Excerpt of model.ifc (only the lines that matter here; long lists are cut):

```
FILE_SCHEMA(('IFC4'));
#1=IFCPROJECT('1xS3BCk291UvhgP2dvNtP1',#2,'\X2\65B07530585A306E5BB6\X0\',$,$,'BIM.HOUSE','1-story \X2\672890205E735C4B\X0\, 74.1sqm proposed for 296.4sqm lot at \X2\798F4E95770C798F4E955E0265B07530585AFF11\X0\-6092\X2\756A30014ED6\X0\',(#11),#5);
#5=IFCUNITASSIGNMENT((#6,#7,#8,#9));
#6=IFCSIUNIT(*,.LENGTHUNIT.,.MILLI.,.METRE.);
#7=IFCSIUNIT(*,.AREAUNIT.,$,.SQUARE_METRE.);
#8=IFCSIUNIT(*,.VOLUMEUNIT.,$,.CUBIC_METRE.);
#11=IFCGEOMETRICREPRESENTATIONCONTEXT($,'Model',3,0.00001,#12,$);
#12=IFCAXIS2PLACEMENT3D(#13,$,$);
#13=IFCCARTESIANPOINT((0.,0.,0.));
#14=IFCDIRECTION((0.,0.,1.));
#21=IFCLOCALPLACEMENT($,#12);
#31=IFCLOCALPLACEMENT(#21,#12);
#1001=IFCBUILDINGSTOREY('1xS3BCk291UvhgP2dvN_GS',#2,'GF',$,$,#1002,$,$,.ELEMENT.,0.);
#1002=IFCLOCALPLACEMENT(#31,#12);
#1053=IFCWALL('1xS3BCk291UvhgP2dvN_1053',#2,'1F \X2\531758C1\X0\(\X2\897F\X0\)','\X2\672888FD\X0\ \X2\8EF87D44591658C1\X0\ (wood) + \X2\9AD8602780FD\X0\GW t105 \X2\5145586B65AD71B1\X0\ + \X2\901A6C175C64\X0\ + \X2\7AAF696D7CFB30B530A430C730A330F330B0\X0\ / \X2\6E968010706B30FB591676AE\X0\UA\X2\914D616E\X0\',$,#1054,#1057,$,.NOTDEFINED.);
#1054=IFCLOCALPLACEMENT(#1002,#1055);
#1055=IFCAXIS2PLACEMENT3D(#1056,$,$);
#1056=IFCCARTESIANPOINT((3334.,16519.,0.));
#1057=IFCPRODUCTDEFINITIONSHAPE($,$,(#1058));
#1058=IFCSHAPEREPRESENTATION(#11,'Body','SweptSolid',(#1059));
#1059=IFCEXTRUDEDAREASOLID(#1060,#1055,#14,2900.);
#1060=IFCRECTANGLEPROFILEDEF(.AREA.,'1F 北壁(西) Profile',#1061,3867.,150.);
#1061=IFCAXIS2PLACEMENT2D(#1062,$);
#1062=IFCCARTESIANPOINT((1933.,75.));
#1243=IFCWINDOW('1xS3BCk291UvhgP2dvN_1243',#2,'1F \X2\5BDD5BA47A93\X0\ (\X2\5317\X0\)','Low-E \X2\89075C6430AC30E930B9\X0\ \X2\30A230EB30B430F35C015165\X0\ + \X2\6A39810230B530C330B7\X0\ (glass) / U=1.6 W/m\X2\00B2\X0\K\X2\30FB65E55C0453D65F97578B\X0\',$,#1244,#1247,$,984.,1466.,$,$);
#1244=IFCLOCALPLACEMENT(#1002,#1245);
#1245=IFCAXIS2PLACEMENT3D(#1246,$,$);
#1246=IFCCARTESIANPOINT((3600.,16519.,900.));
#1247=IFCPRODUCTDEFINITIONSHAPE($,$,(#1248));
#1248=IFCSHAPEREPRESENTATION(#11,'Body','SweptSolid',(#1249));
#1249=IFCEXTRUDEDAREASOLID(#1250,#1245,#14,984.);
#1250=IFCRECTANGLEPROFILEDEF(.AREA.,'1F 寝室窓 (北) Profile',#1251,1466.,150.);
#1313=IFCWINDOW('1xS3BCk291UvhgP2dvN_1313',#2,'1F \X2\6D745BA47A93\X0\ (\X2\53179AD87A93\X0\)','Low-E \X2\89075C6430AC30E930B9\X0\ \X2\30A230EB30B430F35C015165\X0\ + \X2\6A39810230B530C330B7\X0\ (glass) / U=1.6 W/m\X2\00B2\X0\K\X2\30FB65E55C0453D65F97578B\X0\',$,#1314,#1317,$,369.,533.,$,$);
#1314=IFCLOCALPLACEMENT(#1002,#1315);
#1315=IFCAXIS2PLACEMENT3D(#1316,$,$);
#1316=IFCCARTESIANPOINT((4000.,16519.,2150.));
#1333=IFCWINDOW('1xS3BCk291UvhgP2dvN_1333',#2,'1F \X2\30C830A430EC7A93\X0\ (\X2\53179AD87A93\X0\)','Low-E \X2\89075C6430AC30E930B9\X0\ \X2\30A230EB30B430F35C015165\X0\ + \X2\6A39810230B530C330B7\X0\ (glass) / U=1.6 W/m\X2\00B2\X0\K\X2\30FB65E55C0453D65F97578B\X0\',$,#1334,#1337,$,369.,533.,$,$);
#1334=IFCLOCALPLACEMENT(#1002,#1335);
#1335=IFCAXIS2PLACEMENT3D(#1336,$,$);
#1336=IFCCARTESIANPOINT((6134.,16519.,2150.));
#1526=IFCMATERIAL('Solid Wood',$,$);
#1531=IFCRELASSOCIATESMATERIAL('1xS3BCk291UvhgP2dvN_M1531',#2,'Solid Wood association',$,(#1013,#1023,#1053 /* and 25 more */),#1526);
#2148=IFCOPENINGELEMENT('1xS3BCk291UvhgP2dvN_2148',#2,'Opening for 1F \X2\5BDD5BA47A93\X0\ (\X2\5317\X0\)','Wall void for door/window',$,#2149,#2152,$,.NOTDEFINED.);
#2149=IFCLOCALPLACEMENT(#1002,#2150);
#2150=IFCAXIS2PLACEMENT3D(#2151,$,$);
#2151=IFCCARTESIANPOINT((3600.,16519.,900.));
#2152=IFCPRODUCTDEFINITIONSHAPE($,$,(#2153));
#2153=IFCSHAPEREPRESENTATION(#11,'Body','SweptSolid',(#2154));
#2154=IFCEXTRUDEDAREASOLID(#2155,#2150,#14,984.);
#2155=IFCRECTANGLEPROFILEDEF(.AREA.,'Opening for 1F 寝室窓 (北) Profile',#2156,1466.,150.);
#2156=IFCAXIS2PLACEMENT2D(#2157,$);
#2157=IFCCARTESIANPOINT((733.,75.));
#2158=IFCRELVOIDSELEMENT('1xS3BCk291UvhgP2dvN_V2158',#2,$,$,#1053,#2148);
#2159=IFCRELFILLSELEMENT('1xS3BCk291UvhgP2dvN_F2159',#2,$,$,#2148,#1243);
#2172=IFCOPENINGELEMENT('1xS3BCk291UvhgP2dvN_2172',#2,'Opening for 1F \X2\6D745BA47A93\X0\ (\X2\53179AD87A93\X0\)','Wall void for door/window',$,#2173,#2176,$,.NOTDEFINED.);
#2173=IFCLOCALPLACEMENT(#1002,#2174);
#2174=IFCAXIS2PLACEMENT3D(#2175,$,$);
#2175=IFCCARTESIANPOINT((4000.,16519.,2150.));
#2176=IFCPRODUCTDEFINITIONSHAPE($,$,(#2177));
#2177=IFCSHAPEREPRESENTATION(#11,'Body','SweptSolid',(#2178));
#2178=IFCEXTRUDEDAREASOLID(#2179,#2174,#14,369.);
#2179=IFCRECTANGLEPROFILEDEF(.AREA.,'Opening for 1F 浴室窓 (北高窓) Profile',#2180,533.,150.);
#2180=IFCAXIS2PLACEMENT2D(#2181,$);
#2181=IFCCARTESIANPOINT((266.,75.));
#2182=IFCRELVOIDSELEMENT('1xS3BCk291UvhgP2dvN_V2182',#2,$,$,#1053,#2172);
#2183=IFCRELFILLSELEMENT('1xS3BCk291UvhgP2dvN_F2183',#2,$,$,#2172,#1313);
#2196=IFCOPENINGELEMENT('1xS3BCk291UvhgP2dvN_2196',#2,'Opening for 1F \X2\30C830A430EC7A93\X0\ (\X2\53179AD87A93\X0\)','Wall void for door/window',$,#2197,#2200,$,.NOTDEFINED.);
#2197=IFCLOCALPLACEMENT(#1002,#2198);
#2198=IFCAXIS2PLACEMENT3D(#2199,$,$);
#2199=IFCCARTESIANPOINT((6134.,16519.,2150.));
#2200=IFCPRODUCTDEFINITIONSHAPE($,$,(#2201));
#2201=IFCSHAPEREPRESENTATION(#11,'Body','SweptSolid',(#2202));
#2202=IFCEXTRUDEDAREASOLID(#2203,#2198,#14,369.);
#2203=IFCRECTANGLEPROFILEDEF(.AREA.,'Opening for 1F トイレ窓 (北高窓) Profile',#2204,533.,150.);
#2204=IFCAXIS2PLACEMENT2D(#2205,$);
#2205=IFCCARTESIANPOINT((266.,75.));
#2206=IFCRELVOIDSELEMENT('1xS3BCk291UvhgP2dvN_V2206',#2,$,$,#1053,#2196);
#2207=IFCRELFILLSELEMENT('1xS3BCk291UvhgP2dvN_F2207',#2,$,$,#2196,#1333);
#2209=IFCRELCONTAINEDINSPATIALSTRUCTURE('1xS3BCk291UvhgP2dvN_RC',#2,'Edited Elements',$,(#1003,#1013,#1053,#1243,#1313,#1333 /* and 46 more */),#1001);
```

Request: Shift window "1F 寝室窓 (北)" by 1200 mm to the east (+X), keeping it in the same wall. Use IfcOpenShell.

```python
import ifcopenshell
import ifcopenshell.api.geometry
import ifcopenshell.util.placement

model = ifcopenshell.open("model.ifc")

window = model.by_guid("1xS3BCk291UvhgP2dvN_1243")
opening = window.FillsVoids[0].RelatingOpeningElement
wall = opening.VoidsElements[0].RelatingBuildingElement

wall_matrix = ifcopenshell.util.placement.get_local_placement(wall.ObjectPlacement)
shift = wall_matrix[:3, 0] * 1200.0
before = ifcopenshell.util.placement.get_local_placement(window.ObjectPlacement)[:3, 3].copy()

# The window is not placed relative to its opening, so move both.
for product in (opening, window):
    matrix = ifcopenshell.util.placement.get_local_placement(product.ObjectPlacement)
    matrix[:3, 3] += shift
    ifcopenshell.api.geometry.edit_object_placement(model, product=product, matrix=matrix, is_si=False)

after = ifcopenshell.util.placement.get_local_placement(window.ObjectPlacement)[:3, 3]
print("window moved by", (after - before).round(3) + 0.0)

model.write("model_updated.ifc")
```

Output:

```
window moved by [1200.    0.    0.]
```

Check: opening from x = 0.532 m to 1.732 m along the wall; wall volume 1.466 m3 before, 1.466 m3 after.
